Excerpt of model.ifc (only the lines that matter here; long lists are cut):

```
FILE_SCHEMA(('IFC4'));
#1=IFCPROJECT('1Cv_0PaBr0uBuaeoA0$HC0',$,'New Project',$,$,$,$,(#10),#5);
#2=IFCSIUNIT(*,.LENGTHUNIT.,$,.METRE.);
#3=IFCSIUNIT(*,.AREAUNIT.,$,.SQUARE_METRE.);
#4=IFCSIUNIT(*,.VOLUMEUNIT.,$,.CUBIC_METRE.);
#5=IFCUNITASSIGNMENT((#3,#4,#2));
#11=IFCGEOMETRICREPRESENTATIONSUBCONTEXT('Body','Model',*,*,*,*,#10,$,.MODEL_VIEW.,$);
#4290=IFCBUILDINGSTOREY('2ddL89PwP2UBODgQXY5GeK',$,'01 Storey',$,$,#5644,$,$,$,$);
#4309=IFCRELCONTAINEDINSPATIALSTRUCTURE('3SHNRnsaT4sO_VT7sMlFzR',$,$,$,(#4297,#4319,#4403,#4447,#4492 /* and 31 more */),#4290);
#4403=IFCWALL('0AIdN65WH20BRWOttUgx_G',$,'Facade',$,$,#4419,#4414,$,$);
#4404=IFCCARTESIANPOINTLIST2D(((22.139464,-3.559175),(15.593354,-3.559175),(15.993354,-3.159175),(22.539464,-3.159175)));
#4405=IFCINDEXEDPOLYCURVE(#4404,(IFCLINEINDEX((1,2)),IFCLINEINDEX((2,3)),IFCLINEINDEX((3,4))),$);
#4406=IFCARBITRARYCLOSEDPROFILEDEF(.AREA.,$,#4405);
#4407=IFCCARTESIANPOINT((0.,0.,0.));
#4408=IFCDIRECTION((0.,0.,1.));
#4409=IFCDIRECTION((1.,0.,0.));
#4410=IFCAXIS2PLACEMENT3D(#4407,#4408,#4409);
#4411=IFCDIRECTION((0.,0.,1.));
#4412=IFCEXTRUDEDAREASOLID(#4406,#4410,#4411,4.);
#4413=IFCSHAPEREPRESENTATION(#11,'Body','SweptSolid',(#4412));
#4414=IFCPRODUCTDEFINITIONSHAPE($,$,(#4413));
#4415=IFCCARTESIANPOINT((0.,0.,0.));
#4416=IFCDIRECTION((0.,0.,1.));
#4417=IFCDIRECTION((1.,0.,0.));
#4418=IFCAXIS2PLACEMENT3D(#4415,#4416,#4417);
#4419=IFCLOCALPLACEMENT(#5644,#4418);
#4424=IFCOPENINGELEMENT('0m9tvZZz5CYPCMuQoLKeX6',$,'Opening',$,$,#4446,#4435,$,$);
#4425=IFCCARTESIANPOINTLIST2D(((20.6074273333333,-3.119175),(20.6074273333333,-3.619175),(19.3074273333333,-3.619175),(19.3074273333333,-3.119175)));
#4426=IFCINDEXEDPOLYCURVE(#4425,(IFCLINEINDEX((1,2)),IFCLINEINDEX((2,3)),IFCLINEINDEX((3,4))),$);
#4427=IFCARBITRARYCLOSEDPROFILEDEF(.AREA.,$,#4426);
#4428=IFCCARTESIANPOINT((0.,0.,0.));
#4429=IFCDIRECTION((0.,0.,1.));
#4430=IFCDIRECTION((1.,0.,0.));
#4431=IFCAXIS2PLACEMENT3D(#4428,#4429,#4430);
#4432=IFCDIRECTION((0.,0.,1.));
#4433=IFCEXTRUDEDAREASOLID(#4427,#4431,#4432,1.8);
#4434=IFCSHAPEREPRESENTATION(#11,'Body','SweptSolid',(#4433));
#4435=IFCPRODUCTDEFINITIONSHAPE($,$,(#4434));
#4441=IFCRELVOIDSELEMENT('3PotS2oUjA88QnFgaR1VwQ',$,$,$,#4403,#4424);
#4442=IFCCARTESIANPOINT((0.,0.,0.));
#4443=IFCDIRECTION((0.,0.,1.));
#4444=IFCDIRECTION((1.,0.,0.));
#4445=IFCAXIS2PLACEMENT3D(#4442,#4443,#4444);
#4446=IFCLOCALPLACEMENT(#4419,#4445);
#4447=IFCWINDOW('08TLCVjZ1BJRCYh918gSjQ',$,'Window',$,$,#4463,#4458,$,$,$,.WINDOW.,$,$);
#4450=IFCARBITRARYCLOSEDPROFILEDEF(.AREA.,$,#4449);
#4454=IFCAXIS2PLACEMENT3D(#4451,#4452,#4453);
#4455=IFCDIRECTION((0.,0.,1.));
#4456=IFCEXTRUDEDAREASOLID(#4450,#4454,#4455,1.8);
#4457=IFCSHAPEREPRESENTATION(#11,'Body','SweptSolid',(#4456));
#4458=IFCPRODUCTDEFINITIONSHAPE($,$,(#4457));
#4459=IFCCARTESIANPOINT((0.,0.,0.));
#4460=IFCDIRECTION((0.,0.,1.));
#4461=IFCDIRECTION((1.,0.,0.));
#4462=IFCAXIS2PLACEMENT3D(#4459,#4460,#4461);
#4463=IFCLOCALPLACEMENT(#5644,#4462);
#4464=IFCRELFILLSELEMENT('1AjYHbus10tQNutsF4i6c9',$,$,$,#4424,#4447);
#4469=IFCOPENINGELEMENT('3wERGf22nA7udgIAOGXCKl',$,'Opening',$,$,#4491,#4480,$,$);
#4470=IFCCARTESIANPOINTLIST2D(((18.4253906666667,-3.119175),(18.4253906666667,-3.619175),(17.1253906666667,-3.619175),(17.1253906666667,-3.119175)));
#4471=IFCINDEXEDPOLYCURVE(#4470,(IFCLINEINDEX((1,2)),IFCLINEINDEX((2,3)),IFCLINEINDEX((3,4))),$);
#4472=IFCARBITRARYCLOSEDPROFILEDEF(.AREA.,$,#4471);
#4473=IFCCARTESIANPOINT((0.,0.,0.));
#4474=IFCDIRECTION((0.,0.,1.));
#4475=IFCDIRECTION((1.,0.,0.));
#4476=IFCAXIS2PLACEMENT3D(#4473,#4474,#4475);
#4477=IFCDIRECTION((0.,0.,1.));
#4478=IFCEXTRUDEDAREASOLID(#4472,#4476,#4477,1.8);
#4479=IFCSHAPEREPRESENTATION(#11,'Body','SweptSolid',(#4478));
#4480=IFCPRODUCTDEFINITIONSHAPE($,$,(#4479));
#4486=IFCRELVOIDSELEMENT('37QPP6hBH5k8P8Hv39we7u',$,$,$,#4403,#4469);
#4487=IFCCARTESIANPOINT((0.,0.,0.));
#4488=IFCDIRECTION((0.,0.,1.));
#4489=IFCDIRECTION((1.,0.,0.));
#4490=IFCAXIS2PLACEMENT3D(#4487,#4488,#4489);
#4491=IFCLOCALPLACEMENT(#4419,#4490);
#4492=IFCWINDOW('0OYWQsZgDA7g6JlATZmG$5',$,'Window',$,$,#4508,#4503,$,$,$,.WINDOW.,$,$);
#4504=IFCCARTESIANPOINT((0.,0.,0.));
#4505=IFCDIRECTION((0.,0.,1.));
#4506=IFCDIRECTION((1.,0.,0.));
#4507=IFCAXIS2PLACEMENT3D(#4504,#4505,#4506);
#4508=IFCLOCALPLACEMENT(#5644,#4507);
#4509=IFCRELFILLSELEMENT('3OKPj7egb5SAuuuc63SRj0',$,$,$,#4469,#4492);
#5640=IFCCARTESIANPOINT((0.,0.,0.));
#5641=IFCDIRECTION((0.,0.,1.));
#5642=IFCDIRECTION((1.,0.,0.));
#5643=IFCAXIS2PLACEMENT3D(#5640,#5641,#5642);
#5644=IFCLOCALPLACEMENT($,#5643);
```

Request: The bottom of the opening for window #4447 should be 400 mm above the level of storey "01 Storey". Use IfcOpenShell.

```python
import numpy as np
import ifcopenshell
import ifcopenshell.api.geometry
import ifcopenshell.geom
import ifcopenshell.util.element
import ifcopenshell.util.placement
import ifcopenshell.util.shape
import ifcopenshell.util.unit

model = ifcopenshell.open("model.ifc")
unit_scale = ifcopenshell.util.unit.calculate_unit_scale(model)

window = model.by_id(4447)
opening = window.FillsVoids[0].RelatingOpeningElement
storey = ifcopenshell.util.element.get_container(window, ifc_class="IfcBuildingStorey")
level = ifcopenshell.util.placement.get_local_placement(storey.ObjectPlacement)[2, 3]

# The opening's origin need not be at the sill, so measure its lowest point.
shape = ifcopenshell.geom.create_shape(ifcopenshell.geom.settings(), opening)
bottom = ifcopenshell.util.shape.get_shape_bottom_elevation(shape, shape.geometry) / unit_scale
dz = level + 0.4 - bottom

shift = np.array([0.0, 0.0, dz])
# The window is not placed relative to its opening, so move both.
for product in (opening, window):
    matrix = ifcopenshell.util.placement.get_local_placement(product.ObjectPlacement)
    matrix[:3, 3] += shift
    ifcopenshell.api.geometry.edit_object_placement(model, product=product, matrix=matrix, is_si=False)

print(f"moved by {dz * unit_scale:+.3f} m")

model.write("model_edited.ifc")
```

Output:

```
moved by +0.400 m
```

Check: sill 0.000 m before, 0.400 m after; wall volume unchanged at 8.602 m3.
